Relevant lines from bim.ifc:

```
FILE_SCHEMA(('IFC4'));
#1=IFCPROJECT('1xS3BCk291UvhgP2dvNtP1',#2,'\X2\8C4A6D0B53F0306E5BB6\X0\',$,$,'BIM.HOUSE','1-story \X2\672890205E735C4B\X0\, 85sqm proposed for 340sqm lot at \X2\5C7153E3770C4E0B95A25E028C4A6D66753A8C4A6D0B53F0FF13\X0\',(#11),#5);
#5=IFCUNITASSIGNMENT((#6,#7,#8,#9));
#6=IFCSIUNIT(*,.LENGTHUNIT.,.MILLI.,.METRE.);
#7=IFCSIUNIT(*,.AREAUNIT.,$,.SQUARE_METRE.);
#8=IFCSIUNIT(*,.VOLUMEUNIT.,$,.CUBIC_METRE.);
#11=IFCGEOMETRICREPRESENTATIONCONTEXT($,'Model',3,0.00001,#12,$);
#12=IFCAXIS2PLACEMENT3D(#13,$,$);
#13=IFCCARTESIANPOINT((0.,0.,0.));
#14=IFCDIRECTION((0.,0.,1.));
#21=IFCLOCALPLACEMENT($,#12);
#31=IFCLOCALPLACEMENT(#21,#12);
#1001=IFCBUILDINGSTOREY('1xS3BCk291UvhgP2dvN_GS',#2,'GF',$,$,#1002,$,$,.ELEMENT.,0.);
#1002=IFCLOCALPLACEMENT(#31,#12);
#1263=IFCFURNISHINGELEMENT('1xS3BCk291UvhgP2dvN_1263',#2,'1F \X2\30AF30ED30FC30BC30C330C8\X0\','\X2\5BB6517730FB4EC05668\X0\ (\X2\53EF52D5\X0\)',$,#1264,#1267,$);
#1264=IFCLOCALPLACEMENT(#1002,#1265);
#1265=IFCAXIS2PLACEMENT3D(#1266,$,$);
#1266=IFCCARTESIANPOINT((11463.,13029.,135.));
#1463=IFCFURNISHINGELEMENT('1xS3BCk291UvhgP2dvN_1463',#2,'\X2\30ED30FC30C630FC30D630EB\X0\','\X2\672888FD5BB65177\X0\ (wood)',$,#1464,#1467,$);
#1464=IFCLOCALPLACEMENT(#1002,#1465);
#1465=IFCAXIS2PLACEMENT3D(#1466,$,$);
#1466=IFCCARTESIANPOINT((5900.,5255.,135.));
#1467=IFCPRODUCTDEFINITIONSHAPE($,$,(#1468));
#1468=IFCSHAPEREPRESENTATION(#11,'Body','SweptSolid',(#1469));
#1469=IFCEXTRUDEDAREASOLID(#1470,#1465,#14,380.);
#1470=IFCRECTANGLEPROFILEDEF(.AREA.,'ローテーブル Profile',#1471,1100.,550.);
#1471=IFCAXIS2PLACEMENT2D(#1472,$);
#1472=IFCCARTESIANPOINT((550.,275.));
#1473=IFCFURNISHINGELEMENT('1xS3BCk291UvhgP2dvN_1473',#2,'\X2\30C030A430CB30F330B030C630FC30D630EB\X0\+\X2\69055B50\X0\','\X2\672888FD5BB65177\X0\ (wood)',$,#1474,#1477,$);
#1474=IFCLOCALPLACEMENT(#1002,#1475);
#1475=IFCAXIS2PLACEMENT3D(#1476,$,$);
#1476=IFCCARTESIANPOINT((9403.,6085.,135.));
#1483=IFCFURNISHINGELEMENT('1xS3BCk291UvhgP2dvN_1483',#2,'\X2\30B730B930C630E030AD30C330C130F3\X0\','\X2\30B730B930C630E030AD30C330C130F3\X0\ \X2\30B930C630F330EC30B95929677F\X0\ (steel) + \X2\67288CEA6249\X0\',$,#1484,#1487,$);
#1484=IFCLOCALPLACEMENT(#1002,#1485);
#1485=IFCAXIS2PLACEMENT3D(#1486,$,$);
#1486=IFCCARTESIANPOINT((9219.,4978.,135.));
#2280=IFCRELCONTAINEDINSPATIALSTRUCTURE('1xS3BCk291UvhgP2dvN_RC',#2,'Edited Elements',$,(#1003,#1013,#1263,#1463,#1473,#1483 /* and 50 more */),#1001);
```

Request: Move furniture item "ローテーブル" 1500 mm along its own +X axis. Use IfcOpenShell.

```python
import ifcopenshell
import ifcopenshell.api.geometry
import ifcopenshell.util.placement
import ifcopenshell.util.unit

model = ifcopenshell.open("bim.ifc")
unit_scale = ifcopenshell.util.unit.calculate_unit_scale(model)

item = model.by_id(1463)
matrix = ifcopenshell.util.placement.get_local_placement(item.ObjectPlacement)
matrix[:3, 3] += matrix[:3, 0] * 1.5 / unit_scale
ifcopenshell.api.geometry.edit_object_placement(model, product=item, matrix=matrix, is_si=False)

print(ifcopenshell.util.placement.get_local_placement(item.ObjectPlacement).round(3) + 0.0)

model.write("bim_v2.ifc")
```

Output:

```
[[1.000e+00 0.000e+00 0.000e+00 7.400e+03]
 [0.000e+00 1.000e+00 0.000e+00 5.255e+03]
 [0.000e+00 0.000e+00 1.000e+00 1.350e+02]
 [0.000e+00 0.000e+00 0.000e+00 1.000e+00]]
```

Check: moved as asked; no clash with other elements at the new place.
